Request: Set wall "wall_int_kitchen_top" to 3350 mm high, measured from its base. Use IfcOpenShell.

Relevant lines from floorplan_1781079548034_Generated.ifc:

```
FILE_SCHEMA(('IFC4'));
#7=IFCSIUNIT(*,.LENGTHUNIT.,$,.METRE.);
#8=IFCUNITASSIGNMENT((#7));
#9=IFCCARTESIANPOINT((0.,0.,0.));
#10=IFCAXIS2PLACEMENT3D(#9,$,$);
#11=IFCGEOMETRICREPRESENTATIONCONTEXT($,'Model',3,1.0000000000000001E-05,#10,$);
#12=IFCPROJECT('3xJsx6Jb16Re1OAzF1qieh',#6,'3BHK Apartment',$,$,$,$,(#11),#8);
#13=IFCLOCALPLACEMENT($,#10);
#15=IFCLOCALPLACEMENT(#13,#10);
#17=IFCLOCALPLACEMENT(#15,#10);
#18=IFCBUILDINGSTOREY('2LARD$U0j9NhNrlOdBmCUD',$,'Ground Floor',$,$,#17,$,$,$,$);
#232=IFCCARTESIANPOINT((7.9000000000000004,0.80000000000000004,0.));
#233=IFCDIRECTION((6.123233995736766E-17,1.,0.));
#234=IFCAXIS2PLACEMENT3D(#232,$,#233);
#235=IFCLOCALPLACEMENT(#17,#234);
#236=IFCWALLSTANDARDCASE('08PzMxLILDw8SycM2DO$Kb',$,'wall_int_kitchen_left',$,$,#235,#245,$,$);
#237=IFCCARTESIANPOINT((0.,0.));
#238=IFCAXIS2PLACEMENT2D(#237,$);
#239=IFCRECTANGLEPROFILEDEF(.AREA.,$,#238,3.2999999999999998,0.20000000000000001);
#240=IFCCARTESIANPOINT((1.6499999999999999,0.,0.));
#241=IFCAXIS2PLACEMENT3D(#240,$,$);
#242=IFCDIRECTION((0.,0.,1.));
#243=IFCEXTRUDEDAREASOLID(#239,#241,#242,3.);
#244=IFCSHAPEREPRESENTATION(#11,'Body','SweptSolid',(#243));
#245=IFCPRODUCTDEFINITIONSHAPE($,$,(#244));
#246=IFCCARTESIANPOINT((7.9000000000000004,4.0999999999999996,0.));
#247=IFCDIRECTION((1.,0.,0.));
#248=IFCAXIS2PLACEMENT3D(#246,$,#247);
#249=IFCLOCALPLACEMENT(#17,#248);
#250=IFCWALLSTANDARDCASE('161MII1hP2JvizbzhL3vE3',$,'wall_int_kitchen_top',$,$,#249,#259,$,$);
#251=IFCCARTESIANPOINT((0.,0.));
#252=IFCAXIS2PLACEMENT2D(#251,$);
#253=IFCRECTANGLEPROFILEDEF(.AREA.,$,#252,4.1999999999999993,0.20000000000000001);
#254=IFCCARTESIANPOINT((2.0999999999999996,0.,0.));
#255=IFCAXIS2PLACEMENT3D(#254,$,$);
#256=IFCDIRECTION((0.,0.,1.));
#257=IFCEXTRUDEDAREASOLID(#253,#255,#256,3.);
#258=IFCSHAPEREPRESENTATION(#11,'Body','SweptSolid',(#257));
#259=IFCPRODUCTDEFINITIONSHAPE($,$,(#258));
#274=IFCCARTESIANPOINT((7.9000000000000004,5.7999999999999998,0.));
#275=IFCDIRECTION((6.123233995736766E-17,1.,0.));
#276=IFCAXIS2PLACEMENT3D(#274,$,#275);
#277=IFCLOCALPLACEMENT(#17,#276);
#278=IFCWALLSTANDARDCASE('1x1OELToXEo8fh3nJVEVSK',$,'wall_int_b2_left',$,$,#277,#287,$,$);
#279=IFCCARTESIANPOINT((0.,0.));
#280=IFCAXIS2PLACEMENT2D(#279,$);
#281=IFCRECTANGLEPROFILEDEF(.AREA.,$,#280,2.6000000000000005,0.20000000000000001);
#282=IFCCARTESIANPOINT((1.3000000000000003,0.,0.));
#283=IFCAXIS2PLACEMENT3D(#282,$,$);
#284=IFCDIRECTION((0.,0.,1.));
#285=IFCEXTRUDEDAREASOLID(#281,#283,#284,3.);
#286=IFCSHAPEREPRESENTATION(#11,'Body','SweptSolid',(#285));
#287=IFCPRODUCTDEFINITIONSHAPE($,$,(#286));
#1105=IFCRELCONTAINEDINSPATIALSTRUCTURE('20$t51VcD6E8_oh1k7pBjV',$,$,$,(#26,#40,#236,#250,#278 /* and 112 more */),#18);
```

```python
import ifcopenshell
import ifcopenshell.geom
import ifcopenshell.util.shape
import ifcopenshell.util.unit

model = ifcopenshell.open("floorplan_1781079548034_Generated.ifc")
unit_scale = ifcopenshell.util.unit.calculate_unit_scale(model)
settings = ifcopenshell.geom.settings()


def volume(element):
    """Net volume in cubic metres, openings subtracted."""
    shape = ifcopenshell.geom.create_shape(settings, element)
    return ifcopenshell.util.shape.get_volume(shape.geometry)


wall = model.by_id(250)
before = volume(wall)

body = next(r for r in wall.Representation.Representations if r.RepresentationIdentifier == "Body")
solid = body.Items[0]
old_height = solid.Depth
solid.Depth = 3.35 / unit_scale
after = volume(wall)

print(f"height {old_height:g} -> {solid.Depth:g}, volume {before:.3f} -> {after:.3f} m3")

model.write("floorplan_1781079548034_Generated-out.ifc")
```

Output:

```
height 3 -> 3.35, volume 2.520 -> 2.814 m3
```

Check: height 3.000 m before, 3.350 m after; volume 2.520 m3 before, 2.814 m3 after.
